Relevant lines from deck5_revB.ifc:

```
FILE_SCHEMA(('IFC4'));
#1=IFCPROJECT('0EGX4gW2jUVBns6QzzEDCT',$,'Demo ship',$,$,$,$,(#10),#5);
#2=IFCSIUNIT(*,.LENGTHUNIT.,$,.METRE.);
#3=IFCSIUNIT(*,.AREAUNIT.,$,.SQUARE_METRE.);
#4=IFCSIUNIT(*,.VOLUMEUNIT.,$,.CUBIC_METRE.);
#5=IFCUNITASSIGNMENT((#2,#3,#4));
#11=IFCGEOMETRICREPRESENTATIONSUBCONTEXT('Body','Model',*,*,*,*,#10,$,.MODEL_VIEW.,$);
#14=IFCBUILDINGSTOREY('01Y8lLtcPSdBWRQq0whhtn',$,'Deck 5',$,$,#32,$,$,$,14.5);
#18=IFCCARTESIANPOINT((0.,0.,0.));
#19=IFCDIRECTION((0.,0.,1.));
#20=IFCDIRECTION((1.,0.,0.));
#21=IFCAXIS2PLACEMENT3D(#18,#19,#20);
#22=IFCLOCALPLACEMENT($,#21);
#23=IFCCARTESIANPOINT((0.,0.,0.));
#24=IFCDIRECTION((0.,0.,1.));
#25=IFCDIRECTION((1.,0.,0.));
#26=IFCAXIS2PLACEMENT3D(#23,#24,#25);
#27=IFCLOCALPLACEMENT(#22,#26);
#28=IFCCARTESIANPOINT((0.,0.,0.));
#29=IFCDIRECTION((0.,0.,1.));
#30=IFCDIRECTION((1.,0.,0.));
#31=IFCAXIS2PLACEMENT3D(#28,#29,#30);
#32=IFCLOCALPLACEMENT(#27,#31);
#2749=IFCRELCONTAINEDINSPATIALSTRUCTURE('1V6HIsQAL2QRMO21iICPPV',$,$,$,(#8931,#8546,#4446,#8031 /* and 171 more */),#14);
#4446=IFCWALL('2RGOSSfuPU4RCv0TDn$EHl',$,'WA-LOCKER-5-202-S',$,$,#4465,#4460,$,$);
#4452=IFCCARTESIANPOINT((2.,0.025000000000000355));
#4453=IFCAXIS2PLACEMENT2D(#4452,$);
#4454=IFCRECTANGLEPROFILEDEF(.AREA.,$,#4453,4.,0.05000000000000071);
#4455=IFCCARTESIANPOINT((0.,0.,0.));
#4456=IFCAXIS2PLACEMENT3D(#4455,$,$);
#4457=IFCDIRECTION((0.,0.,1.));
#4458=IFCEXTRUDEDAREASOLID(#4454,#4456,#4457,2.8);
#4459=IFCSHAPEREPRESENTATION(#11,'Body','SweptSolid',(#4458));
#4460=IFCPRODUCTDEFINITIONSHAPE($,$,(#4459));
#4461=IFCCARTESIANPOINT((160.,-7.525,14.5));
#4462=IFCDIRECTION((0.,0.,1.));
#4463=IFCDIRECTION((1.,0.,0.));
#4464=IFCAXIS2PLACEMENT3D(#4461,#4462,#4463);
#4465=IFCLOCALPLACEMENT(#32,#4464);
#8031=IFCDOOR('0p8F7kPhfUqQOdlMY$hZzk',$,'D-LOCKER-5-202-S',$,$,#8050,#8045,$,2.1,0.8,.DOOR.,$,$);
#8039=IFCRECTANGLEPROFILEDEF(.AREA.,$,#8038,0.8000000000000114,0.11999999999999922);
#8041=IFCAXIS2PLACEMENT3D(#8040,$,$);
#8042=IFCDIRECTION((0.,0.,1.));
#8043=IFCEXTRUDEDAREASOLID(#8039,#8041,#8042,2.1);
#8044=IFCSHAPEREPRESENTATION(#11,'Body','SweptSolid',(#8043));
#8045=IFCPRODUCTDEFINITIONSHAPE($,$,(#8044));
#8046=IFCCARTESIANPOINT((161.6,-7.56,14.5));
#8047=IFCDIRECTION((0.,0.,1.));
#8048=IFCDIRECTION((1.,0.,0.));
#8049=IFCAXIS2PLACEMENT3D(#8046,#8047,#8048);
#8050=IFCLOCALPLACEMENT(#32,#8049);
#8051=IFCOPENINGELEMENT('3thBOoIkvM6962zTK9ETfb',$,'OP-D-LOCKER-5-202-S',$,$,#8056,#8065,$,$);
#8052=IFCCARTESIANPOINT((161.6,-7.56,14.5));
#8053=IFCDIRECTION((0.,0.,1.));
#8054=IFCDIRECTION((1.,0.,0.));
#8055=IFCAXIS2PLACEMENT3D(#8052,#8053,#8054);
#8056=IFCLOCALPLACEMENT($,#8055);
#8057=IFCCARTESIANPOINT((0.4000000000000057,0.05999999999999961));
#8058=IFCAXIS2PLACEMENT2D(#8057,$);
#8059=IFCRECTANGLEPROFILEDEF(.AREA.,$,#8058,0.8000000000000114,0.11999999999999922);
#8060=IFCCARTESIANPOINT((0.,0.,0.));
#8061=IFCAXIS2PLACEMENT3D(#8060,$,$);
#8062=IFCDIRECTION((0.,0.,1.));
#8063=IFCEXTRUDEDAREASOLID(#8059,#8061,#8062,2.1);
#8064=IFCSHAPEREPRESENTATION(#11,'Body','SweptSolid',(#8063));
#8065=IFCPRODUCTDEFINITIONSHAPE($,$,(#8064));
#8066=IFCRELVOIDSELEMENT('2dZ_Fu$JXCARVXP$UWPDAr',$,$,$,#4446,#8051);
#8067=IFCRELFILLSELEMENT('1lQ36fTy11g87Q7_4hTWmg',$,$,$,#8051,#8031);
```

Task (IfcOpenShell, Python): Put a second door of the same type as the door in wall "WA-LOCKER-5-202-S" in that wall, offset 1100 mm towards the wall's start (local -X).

```python
import ifcopenshell
import ifcopenshell.api.feature
import ifcopenshell.api.geometry
import ifcopenshell.api.root
import ifcopenshell.geom
import ifcopenshell.util.element
import ifcopenshell.util.placement
import ifcopenshell.util.shape
import ifcopenshell.util.unit

model = ifcopenshell.open("deck5_revB.ifc")
unit_scale = ifcopenshell.util.unit.calculate_unit_scale(model)
settings = ifcopenshell.geom.settings()


def volume(element):
    """Net volume in cubic metres, openings subtracted."""
    shape = ifcopenshell.geom.create_shape(settings, element)
    return ifcopenshell.util.shape.get_volume(shape.geometry)


door = model.by_guid("0p8F7kPhfUqQOdlMY$hZzk")
opening = door.FillsVoids[0].RelatingOpeningElement
wall = opening.VoidsElements[0].RelatingBuildingElement
before = volume(wall)
shift = ifcopenshell.util.placement.get_local_placement(wall.ObjectPlacement)[:3, 0] * -1.1 / unit_scale

# copy_class copies the void relationship, type, container and properties, but no geometry.
new_opening = ifcopenshell.api.root.copy_class(model, product=opening)
new_opening.Representation = ifcopenshell.util.element.copy_deep(
    model, opening.Representation, exclude=["IfcGeometricRepresentationContext", "IfcRepresentationMap"]
)
new_door = ifcopenshell.api.root.copy_class(model, product=door)
new_door.Representation = ifcopenshell.util.element.copy_deep(
    model, door.Representation, exclude=["IfcGeometricRepresentationContext", "IfcRepresentationMap"]
)
ifcopenshell.api.feature.add_filling(model, opening=new_opening, element=new_door)

for old, new in ((opening, new_opening), (door, new_door)):
    matrix = ifcopenshell.util.placement.get_local_placement(old.ObjectPlacement)
    matrix[:3, 3] += shift
    ifcopenshell.api.geometry.edit_object_placement(model, product=new, matrix=matrix, is_si=False)

after = volume(wall)

print(f"wall volume {before:.3f} -> {after:.3f} m3")

model.write("deck5_revB_rev.ifc")
```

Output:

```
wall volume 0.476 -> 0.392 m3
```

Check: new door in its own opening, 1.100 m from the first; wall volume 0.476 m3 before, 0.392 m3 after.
